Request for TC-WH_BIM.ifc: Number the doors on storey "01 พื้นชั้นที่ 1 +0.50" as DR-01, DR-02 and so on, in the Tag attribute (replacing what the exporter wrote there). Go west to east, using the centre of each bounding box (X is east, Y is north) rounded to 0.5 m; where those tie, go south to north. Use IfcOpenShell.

First a look at what the model holds.

```python
import ifcopenshell
import ifcopenshell.util.element
import ifcopenshell.util.placement

model = ifcopenshell.open("TC-WH_BIM.ifc")
print(model.schema)
storey = next(s for s in model.by_type("IfcBuildingStorey") if s.Name == "01 พื้นชั้นที่ 1 +0.50")
doors = [e for e in ifcopenshell.util.element.get_decomposition(storey) if e.is_a("IfcDoor")]
for e in sorted(doors, key=lambda e: e.id()):
    origin = ifcopenshell.util.placement.get_local_placement(e.ObjectPlacement)[:3, 3]
    print(e.id(), e.Tag, e.Name, origin.round(2) + 0.0, sep=" | ")
```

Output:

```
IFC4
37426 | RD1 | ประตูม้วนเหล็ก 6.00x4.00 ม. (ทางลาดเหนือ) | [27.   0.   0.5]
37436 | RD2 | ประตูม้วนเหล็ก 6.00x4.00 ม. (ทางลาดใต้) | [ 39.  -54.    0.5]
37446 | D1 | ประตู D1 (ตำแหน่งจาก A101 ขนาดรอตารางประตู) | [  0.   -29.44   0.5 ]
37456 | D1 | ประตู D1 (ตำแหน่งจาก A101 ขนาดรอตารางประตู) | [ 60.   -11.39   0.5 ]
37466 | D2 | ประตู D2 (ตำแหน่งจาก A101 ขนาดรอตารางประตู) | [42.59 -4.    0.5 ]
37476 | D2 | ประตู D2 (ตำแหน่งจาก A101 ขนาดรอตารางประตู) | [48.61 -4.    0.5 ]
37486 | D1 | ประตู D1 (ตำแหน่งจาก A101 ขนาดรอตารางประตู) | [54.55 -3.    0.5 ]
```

```python
import ifcopenshell
import ifcopenshell.geom
import ifcopenshell.util.element
import ifcopenshell.util.shape

model = ifcopenshell.open("TC-WH_BIM.ifc")
settings = ifcopenshell.geom.settings()
settings.set("use-world-coords", True)


def centre(element):
    shape = ifcopenshell.geom.create_shape(settings, element)
    return ifcopenshell.util.shape.get_bbox_centroid(shape.geometry)


storey = next(s for s in model.by_type("IfcBuildingStorey") if s.Name == "01 พื้นชั้นที่ 1 +0.50")
doors = [e for e in ifcopenshell.util.element.get_decomposition(storey) if e.is_a("IfcDoor")]

# Insertion points can sit at a corner or the storey origin, so sort by the geometry (in metres).
centres = {e: centre(e) for e in doors}
doors.sort(key=lambda e: (round(centres[e][0] / 0.5), centres[e][1]))

for i, e in enumerate(doors, start=1):
    number = f"DR-{i:02d}"
    e.Tag = number
    print(e.id(), number)

model.write("TC-WH_BIM_updated.ifc")
```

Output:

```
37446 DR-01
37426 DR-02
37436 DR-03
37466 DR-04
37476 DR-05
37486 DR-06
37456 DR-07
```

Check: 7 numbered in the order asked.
